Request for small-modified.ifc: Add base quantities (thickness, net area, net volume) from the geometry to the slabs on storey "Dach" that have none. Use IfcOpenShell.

First a look at what the model holds.

```python
import ifcopenshell
import ifcopenshell.util.element
import ifcopenshell.util.unit

model = ifcopenshell.open("small-modified.ifc")
print(model.schema)
for unit_type in ("LENGTHUNIT", "AREAUNIT", "VOLUMEUNIT"):
    print(unit_type, ifcopenshell.util.unit.calculate_unit_scale(model, unit_type))
storey = next(s for s in model.by_type("IfcBuildingStorey") if s.Name == "Dach")
slabs = [e for e in ifcopenshell.util.element.get_decomposition(storey) if e.is_a("IfcSlab")]
for e in sorted(slabs, key=lambda e: e.id()):
    print(e.id(), e.is_a(), e.Name, list(ifcopenshell.util.element.get_psets(e, qtos_only=True)), sep=" | ")
```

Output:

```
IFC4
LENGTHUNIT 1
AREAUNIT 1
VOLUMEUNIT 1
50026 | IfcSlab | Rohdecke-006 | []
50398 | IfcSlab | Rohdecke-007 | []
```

```python
import ifcopenshell
import ifcopenshell.api.pset
import ifcopenshell.geom
import ifcopenshell.util.element
import ifcopenshell.util.shape
import ifcopenshell.util.unit

model = ifcopenshell.open("small-modified.ifc")
unit_scale = ifcopenshell.util.unit.calculate_unit_scale(model)
area_scale = ifcopenshell.util.unit.calculate_unit_scale(model, "AREAUNIT")
volume_scale = ifcopenshell.util.unit.calculate_unit_scale(model, "VOLUMEUNIT")
settings = ifcopenshell.geom.settings()

storey = next(s for s in model.by_type("IfcBuildingStorey") if s.Name == "Dach")
slabs = [e for e in ifcopenshell.util.element.get_decomposition(storey) if e.is_a("IfcSlab")]

for e in sorted(slabs, key=lambda e: e.id()):
    if ifcopenshell.util.element.get_psets(e, qtos_only=True, should_inherit=False):
        continue
    # Geometry comes back in metres, in the element's own axes.
    shape = ifcopenshell.geom.create_shape(settings, e)
    values = {
        "Width": ifcopenshell.util.shape.get_z(shape.geometry) / unit_scale,
        "NetArea": ifcopenshell.util.shape.get_footprint_area(shape.geometry) / area_scale,
        "NetVolume": ifcopenshell.util.shape.get_volume(shape.geometry) / volume_scale,
    }
    qto = ifcopenshell.api.pset.add_qto(model, product=e, name="Qto_SlabBaseQuantities")
    ifcopenshell.api.pset.edit_qto(model, qto=qto, properties=values)
    print(e.id(), {k: round(v, 3) for k, v in values.items()})

model.write("small-modified_rev.ifc")
```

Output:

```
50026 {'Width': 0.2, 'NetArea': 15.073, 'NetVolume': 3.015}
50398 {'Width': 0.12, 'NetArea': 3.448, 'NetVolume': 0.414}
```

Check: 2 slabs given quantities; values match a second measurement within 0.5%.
